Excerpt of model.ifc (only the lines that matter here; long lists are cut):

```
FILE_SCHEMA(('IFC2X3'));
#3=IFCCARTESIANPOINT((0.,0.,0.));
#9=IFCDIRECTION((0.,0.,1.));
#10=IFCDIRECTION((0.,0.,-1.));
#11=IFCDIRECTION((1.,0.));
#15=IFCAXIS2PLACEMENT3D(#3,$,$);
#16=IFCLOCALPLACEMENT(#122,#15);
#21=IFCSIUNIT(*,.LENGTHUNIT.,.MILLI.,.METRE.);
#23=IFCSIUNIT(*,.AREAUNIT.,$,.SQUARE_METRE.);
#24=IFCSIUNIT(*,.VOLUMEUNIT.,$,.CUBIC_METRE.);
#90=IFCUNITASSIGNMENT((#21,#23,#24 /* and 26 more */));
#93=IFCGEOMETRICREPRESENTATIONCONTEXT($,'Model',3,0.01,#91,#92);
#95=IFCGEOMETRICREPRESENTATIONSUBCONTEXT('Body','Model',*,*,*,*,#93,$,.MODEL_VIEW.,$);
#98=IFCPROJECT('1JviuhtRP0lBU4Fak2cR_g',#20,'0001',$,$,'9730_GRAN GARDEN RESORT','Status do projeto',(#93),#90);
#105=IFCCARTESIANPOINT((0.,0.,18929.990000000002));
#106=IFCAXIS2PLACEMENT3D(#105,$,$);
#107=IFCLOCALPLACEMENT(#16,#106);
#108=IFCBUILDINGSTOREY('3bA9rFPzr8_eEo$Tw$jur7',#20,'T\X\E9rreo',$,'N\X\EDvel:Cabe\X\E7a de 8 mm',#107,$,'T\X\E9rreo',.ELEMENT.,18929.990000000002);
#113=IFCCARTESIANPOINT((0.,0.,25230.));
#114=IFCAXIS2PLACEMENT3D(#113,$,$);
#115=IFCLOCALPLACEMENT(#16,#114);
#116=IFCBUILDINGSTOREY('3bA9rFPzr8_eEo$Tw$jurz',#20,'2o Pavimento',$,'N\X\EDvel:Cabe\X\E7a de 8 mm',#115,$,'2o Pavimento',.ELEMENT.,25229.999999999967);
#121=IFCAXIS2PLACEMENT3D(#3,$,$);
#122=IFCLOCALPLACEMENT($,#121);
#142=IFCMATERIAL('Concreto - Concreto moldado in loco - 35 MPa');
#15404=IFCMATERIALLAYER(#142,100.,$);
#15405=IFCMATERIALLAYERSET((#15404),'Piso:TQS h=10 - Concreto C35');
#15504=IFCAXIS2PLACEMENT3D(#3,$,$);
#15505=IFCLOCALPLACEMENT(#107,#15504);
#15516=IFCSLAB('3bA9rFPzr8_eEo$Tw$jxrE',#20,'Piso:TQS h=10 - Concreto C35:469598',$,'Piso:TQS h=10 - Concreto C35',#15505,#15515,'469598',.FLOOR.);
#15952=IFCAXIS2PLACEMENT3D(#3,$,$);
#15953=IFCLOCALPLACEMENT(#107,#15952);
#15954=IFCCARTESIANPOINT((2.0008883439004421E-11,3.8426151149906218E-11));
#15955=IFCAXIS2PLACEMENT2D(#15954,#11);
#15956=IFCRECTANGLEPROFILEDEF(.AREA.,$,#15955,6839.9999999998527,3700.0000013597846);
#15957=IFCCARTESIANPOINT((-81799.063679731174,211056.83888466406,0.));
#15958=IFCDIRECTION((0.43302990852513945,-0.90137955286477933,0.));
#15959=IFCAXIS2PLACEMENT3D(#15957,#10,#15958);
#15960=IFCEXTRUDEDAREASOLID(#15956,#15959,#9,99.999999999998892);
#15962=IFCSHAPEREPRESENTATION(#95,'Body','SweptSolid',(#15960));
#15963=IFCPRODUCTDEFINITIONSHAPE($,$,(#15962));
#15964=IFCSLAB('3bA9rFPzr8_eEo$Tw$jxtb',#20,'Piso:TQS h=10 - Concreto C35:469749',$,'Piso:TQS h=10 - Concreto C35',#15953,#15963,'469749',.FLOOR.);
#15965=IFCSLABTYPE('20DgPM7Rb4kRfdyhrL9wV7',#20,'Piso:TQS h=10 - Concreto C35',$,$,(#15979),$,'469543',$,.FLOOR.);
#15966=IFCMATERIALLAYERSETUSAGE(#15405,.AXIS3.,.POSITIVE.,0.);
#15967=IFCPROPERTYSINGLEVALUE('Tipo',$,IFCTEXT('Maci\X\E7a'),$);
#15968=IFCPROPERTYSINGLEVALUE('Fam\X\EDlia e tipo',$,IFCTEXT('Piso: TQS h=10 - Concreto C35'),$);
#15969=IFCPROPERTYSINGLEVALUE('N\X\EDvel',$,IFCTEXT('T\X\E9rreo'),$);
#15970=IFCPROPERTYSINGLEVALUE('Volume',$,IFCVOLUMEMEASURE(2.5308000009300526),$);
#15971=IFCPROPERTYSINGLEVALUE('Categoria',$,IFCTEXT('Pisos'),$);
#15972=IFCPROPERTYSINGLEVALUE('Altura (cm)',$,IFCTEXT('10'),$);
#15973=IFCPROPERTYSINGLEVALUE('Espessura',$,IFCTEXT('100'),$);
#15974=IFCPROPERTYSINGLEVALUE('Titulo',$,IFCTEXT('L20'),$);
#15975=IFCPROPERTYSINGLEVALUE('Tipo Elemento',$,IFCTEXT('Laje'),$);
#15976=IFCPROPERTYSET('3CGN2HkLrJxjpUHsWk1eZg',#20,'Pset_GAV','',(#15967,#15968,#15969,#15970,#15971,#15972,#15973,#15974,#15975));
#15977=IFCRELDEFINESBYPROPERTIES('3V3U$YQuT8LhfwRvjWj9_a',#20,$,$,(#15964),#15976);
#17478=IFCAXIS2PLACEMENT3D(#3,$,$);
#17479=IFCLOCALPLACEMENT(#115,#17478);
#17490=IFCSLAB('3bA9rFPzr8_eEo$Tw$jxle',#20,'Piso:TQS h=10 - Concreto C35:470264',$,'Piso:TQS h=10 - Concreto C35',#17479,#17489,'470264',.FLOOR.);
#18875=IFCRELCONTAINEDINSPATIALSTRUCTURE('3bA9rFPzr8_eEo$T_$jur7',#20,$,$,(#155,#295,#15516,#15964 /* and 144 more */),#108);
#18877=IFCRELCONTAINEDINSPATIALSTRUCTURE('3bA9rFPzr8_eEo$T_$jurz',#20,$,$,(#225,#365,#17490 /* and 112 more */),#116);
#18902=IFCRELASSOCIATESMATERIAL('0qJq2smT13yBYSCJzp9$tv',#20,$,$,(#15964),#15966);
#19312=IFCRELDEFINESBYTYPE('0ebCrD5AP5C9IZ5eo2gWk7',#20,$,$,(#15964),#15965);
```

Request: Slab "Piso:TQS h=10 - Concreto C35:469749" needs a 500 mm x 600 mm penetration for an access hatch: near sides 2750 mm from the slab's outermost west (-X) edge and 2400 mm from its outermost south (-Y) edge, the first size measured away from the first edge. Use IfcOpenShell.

```python
import numpy as np
import ifcopenshell
import ifcopenshell.api.feature
import ifcopenshell.api.geometry
import ifcopenshell.api.pset
import ifcopenshell.api.root
import ifcopenshell.geom
import ifcopenshell.util.element
import ifcopenshell.util.placement
import ifcopenshell.util.representation
import ifcopenshell.util.shape
import ifcopenshell.util.unit

model = ifcopenshell.open("model.ifc")
unit_scale = ifcopenshell.util.unit.calculate_unit_scale(model)
volume_scale = ifcopenshell.util.unit.calculate_unit_scale(model, "VOLUMEUNIT")
settings = ifcopenshell.geom.settings()


def volume(element):
    """Net volume in cubic metres, openings subtracted."""
    shape = ifcopenshell.geom.create_shape(settings, element)
    return ifcopenshell.util.shape.get_volume(shape.geometry)


slab = model.by_guid("3bA9rFPzr8_eEo$Tw$jxtb")
before = volume(slab)

# Extent in the slab's own axes, in metres. The edges named are its -X and -Y sides.
slab_shape = ifcopenshell.geom.create_shape(settings, slab)
vertices = ifcopenshell.util.shape.get_vertices(slab_shape.geometry)
x_min, y_min, bottom = vertices.min(axis=0)
top = vertices[:, 2].max()

opening = ifcopenshell.api.root.create_entity(model, ifc_class="IfcOpeningElement", name="Access hatch opening")
context = ifcopenshell.util.representation.get_context(model, "Model", "Body", "MODEL_VIEW")
width, depth = 0.5, 0.6
outline = [(0.0, 0.0), (width, 0.0), (width, depth), (0.0, depth), (0.0, 0.0)]
# Overshoot both faces by 50 mm so the cut is clean.
shape = ifcopenshell.api.geometry.add_slab_representation(
    model, context=context, depth=top - bottom + 0.1, polyline=outline
)
ifcopenshell.api.geometry.assign_representation(model, product=opening, representation=shape)

matrix = ifcopenshell.util.placement.get_local_placement(slab.ObjectPlacement)
matrix[:, 3] = matrix @ np.append(np.array([x_min + 2.75, y_min + 2.4, bottom - 0.05]) / unit_scale, 1.0)
ifcopenshell.api.geometry.edit_object_placement(model, product=opening, matrix=matrix, is_si=False)
ifcopenshell.api.feature.add_feature(model, feature=opening, element=slab)

after = volume(slab)

# Update the slab's stored quantities.
pset = model.by_id(ifcopenshell.util.element.get_pset(slab, "Pset_GAV", should_inherit=False)["id"])
ifcopenshell.api.pset.edit_pset(model, pset=pset, properties={
    "Volume": model.create_entity("IfcVolumeMeasure", after / volume_scale),
})

print(f"slab volume {before:.3f} -> {after:.3f} m3")

model.write("model_updated.ifc")
```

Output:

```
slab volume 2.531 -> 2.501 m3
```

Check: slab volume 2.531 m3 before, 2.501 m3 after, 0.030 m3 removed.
